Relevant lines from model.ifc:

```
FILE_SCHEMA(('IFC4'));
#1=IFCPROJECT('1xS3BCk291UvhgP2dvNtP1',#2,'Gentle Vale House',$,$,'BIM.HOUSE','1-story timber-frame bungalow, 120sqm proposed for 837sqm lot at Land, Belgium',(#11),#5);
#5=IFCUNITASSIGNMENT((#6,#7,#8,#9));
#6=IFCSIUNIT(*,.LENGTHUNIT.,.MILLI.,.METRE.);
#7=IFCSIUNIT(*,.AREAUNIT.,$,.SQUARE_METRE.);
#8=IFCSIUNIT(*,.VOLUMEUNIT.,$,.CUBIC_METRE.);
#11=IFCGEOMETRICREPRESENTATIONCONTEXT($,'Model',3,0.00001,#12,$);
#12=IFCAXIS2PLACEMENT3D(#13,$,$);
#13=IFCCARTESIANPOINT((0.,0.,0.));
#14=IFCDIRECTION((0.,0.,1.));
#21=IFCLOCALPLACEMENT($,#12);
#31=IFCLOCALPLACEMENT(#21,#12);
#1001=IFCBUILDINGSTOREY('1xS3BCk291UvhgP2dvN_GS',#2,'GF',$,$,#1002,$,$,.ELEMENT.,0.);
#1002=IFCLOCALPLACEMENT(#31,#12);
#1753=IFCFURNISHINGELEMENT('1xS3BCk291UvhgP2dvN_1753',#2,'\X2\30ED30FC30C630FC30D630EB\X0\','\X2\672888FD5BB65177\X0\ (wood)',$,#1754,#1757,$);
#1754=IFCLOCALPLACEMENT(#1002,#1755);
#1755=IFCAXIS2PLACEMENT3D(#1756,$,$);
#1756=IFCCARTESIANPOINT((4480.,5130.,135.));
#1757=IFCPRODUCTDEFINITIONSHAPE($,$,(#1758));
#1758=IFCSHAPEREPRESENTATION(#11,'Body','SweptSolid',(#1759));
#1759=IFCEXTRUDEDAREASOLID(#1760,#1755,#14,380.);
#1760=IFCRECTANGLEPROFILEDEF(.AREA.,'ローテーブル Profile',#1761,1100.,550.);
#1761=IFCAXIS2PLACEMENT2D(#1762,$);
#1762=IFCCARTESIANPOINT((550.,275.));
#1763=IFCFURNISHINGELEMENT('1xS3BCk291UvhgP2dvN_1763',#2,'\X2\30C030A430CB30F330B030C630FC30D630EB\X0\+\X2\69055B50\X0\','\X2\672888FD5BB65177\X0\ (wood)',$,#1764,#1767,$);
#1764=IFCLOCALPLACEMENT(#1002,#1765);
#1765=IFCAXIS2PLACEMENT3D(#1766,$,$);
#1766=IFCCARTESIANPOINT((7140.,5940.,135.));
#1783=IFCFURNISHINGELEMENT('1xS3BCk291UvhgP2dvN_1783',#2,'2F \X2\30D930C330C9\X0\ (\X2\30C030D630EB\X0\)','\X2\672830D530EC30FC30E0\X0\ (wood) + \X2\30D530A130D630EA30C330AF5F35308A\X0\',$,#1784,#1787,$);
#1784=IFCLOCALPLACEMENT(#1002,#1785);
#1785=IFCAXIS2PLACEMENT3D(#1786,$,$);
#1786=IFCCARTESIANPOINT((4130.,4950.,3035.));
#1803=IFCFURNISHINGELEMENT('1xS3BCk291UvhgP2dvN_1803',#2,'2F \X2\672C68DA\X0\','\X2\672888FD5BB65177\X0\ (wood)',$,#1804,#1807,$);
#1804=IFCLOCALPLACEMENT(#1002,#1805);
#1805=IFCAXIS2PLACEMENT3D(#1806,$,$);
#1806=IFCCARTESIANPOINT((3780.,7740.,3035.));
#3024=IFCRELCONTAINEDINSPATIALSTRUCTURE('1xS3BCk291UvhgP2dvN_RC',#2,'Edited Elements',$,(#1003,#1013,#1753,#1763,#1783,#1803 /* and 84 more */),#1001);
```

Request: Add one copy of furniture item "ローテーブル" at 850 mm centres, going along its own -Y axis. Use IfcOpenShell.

```python
import ifcopenshell
import ifcopenshell.api.geometry
import ifcopenshell.api.root
import ifcopenshell.util.element
import ifcopenshell.util.placement
import ifcopenshell.util.unit

model = ifcopenshell.open("model.ifc")
unit_scale = ifcopenshell.util.unit.calculate_unit_scale(model)


def reuse_history(source, copy):
    """copy_class also copies each property set's owner history, people and application; keep the originals."""
    for rel in copy.IsDefinedBy:
        if rel.is_a("IfcRelDefinesByProperties") and (history := rel.RelatingPropertyDefinition.OwnerHistory):
            rel.RelatingPropertyDefinition.OwnerHistory = source.OwnerHistory
            ifcopenshell.util.element.remove_deep2(model, history)


source = model.by_guid("1xS3BCk291UvhgP2dvN_1753")
base = ifcopenshell.util.placement.get_local_placement(source.ObjectPlacement)
step = -base[:3, 1] * 0.85 / unit_scale

for i in range(1, 2):
    copy = ifcopenshell.api.root.copy_class(model, product=source)
    copy.Representation = ifcopenshell.util.element.copy_deep(
        model, source.Representation, exclude=["IfcGeometricRepresentationContext", "IfcRepresentationMap"]
    )
    reuse_history(source, copy)
    matrix = base.copy()
    matrix[:3, 3] += i * step
    print("added at", matrix[:3, 3].round(3) + 0.0)
    ifcopenshell.api.geometry.edit_object_placement(model, product=copy, matrix=matrix, is_si=False)

model.write("model_rev.ifc")
```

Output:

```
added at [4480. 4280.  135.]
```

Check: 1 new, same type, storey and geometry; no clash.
